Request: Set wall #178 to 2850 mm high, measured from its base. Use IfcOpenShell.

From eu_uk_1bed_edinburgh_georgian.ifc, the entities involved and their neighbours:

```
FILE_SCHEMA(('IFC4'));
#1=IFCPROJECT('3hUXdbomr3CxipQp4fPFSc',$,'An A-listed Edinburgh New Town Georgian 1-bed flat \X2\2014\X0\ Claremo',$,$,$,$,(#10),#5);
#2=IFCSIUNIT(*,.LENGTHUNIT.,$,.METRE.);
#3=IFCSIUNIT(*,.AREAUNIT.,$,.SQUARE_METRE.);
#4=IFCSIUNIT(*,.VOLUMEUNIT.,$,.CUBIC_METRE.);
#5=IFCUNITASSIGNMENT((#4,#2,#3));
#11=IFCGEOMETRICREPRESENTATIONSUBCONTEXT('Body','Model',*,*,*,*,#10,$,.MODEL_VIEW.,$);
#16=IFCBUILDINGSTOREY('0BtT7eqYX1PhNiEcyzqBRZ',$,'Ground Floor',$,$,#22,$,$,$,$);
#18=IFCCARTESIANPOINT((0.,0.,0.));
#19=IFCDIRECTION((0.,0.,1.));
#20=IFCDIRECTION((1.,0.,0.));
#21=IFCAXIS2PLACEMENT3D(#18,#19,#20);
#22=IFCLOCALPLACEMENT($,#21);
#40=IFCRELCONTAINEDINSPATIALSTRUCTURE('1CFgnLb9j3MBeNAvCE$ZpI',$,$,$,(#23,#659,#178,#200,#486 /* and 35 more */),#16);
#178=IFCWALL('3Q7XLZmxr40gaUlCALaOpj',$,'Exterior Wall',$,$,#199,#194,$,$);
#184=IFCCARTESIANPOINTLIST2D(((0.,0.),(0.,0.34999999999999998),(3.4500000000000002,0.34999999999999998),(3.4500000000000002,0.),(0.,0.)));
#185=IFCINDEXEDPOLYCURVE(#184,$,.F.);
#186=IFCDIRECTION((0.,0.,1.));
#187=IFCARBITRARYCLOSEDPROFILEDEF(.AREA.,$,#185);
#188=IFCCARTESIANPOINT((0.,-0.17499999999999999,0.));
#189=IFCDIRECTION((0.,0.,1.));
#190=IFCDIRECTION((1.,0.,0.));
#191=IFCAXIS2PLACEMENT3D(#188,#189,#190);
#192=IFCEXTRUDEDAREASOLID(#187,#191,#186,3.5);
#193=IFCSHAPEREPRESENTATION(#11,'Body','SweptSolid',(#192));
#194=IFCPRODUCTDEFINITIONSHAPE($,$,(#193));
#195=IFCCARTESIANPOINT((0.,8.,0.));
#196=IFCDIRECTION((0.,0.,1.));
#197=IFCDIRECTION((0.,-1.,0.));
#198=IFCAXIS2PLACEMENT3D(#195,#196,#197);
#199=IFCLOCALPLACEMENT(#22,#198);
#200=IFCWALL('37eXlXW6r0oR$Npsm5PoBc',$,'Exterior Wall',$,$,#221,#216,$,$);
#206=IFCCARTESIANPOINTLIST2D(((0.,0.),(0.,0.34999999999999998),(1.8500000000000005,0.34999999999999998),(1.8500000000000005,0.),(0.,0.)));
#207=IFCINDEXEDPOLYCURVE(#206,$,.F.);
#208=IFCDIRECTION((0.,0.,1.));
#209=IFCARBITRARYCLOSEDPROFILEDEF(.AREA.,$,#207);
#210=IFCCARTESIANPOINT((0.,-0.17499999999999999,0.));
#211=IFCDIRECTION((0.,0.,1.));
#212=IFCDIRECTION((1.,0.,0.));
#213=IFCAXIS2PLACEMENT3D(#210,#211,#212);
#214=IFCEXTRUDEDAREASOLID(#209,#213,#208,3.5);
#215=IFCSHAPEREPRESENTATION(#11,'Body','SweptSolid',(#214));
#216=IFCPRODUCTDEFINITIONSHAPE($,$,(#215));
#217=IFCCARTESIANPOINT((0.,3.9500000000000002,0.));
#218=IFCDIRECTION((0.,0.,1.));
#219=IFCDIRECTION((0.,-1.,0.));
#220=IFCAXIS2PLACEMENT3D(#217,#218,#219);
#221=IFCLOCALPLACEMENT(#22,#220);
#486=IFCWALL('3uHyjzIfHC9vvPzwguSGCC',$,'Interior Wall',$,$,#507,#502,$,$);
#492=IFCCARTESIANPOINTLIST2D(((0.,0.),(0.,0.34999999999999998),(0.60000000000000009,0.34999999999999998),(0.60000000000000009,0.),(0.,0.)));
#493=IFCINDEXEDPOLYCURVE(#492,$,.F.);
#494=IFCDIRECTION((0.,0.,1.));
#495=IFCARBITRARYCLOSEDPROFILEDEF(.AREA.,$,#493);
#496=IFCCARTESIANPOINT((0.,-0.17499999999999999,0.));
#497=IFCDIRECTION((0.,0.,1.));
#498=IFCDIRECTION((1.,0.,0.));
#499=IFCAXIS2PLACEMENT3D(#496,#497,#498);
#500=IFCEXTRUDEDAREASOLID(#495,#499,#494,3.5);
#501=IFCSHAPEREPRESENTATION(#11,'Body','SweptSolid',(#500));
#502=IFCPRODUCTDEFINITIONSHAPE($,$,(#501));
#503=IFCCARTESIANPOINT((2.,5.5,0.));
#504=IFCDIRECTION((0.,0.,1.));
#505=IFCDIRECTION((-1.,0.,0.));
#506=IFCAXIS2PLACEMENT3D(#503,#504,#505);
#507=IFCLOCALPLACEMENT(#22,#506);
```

```python
import ifcopenshell
import ifcopenshell.geom
import ifcopenshell.util.representation
import ifcopenshell.util.shape

model = ifcopenshell.open("eu_uk_1bed_edinburgh_georgian.ifc")
settings = ifcopenshell.geom.settings()


def volume(element):
    """Net volume in cubic metres, openings subtracted."""
    shape = ifcopenshell.geom.create_shape(settings, element)
    return ifcopenshell.util.shape.get_volume(shape.geometry)


wall = model.by_guid("3Q7XLZmxr40gaUlCALaOpj")
before = volume(wall)

body = ifcopenshell.util.representation.get_representation(wall, "Model", "Body")
solid = body.Items[0]
old_height = solid.Depth
solid.Depth = 2.85
after = volume(wall)

print(f"height {old_height:g} -> {solid.Depth:g}, volume {before:.3f} -> {after:.3f} m3")

model.write("eu_uk_1bed_edinburgh_georgian_updated.ifc")
```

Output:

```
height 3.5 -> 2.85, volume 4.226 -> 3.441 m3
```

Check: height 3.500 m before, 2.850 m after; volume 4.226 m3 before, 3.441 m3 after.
